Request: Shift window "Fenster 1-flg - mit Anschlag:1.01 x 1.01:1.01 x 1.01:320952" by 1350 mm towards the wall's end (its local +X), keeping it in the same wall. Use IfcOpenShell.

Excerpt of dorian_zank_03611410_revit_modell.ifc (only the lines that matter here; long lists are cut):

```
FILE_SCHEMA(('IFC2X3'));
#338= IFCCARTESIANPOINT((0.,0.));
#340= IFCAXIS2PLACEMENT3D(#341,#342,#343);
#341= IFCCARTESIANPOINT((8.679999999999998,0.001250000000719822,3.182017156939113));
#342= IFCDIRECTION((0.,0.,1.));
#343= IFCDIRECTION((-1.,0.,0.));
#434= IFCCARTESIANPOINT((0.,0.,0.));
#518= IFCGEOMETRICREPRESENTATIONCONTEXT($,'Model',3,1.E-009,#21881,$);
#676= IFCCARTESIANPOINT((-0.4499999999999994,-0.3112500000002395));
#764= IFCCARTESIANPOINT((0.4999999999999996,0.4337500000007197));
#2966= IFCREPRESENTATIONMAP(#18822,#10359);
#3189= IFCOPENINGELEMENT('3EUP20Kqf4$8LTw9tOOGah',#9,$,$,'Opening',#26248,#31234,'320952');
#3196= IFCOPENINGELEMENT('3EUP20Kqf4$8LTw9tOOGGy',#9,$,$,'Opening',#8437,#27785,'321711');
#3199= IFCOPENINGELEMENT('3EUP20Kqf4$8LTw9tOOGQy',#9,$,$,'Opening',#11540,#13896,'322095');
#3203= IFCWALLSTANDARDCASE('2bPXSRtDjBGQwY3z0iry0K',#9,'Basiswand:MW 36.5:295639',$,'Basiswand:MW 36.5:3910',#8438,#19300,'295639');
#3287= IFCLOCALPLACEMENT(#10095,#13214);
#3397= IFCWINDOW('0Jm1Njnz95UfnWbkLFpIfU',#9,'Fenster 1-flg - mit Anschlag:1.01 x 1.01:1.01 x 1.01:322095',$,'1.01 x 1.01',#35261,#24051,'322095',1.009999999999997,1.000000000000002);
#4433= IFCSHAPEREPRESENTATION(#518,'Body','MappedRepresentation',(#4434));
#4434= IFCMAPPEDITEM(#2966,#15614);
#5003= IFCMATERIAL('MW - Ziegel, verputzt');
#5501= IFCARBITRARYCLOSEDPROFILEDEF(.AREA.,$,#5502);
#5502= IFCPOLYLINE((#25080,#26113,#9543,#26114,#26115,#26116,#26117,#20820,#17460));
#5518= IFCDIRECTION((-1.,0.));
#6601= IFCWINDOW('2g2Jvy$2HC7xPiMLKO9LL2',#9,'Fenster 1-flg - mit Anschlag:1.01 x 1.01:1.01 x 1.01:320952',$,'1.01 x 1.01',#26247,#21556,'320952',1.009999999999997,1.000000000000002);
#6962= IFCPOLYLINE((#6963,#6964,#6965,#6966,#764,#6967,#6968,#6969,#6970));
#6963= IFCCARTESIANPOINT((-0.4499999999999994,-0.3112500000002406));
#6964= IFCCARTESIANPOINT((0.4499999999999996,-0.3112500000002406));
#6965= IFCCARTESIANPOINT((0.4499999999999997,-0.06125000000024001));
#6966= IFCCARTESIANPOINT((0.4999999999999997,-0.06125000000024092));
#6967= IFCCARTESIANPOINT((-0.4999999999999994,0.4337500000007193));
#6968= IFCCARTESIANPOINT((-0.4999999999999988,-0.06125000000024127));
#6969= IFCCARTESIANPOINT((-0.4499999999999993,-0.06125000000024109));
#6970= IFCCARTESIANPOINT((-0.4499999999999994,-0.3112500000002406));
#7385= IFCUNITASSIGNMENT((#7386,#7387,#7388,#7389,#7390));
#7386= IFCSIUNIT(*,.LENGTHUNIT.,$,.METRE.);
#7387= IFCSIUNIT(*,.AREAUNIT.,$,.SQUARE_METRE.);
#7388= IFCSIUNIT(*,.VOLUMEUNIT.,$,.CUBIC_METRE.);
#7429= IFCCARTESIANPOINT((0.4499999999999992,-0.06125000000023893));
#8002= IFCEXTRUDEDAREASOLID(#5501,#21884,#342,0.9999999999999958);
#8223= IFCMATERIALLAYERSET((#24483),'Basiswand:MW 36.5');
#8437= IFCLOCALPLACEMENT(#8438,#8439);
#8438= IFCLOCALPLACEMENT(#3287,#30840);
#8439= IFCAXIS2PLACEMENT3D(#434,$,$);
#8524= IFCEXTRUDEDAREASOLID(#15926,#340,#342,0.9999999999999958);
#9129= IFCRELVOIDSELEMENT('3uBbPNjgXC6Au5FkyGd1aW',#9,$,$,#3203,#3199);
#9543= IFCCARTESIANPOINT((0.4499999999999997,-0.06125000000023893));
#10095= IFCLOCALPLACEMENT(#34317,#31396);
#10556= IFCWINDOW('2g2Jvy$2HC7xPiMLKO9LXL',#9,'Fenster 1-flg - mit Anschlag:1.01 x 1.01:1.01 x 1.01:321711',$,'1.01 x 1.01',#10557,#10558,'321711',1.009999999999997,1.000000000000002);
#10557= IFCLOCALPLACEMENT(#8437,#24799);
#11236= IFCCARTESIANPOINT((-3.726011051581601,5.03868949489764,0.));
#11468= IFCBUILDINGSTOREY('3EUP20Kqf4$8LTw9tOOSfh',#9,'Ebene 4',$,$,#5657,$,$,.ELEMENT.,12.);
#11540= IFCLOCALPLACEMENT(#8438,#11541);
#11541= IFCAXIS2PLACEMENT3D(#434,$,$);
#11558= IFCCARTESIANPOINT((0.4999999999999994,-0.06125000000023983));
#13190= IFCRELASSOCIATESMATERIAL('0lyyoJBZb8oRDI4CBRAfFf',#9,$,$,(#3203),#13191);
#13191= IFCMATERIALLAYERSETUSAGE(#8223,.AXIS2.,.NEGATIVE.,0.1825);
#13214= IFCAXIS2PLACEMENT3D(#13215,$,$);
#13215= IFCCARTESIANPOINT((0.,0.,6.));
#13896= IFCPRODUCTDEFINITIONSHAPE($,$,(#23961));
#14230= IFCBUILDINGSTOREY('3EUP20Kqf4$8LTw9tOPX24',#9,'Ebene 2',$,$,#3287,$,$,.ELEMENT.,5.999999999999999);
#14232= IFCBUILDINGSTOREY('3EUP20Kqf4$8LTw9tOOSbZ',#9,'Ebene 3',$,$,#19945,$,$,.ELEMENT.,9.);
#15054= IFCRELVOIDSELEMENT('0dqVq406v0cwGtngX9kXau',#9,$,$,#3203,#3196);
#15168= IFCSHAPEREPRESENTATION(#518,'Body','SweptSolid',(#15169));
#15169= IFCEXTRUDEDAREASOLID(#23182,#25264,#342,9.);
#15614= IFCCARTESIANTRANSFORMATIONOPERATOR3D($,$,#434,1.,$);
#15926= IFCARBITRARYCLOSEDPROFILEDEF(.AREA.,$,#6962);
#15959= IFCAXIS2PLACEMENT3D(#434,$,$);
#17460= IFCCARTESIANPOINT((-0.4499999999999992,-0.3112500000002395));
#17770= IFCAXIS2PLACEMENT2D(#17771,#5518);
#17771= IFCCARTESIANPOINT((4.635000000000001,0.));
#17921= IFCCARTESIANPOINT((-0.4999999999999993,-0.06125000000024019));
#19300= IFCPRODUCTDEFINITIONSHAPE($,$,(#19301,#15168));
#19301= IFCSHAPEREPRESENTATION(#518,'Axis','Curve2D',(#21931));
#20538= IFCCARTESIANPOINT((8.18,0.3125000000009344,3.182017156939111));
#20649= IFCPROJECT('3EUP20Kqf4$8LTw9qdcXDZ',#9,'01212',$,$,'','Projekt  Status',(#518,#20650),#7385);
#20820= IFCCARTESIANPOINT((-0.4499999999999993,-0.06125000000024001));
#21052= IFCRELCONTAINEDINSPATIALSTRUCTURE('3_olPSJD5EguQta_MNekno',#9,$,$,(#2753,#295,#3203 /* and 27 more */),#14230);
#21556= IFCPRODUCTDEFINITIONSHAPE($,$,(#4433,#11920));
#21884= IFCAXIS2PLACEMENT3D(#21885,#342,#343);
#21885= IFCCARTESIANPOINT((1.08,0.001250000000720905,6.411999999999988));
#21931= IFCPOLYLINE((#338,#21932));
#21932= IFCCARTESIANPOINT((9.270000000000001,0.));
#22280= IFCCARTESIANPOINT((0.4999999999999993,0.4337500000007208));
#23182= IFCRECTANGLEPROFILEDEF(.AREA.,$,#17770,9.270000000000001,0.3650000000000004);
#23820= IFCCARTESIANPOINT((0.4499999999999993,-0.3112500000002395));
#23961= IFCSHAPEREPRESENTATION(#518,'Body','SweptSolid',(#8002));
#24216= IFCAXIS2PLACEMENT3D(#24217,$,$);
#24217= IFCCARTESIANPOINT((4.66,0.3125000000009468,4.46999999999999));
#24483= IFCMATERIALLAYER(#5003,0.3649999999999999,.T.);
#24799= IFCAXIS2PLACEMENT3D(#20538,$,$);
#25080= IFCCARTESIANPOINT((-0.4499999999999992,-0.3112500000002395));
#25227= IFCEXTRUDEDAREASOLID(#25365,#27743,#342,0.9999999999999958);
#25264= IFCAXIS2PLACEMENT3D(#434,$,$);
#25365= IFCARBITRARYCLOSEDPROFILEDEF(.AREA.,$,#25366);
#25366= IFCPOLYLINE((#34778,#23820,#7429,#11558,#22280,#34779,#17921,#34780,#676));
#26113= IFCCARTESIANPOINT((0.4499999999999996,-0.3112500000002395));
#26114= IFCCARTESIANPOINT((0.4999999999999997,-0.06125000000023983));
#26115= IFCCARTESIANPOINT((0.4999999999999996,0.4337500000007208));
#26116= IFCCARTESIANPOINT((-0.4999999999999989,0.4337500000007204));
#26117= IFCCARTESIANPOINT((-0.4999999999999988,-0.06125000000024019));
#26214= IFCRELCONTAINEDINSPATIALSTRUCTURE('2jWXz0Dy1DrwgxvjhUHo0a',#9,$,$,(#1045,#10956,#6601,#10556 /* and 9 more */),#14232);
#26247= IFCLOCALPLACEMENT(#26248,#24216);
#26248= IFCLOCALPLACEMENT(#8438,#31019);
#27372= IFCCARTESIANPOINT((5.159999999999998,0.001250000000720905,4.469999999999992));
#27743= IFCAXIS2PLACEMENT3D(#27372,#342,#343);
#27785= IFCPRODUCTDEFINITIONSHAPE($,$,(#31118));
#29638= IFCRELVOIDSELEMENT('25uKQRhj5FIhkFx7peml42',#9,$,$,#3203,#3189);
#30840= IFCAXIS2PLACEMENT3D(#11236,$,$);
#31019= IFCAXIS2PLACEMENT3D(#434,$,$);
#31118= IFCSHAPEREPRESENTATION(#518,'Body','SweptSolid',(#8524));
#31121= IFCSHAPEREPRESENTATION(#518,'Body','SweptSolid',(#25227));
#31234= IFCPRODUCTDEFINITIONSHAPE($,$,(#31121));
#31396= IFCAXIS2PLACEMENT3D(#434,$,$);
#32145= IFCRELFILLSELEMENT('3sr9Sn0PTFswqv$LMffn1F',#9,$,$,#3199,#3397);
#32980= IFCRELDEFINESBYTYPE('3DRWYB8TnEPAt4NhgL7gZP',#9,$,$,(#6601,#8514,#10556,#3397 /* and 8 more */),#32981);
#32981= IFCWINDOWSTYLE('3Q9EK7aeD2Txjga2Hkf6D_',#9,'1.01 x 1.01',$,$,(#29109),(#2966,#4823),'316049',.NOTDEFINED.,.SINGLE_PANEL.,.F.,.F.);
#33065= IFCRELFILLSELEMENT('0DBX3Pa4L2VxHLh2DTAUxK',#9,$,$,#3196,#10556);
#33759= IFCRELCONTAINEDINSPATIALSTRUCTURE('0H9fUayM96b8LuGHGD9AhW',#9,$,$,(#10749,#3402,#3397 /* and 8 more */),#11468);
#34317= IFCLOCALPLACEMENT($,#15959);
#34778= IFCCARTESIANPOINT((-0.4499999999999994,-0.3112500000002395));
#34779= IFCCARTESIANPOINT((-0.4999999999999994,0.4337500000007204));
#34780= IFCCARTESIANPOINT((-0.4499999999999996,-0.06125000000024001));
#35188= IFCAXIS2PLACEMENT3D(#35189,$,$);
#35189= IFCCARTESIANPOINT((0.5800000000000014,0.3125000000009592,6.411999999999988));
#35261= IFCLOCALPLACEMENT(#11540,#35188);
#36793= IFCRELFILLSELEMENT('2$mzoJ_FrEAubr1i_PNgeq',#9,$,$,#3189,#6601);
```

```python
import ifcopenshell
import ifcopenshell.api.geometry
import ifcopenshell.util.placement
import ifcopenshell.util.unit

model = ifcopenshell.open("dorian_zank_03611410_revit_modell.ifc")
unit_scale = ifcopenshell.util.unit.calculate_unit_scale(model)

window = model.by_guid("2g2Jvy$2HC7xPiMLKO9LL2")
opening = window.FillsVoids[0].RelatingOpeningElement
wall = opening.VoidsElements[0].RelatingBuildingElement

wall_matrix = ifcopenshell.util.placement.get_local_placement(wall.ObjectPlacement)
shift = wall_matrix[:3, 0] * 1.35 / unit_scale
before = ifcopenshell.util.placement.get_local_placement(window.ObjectPlacement)[:3, 3].copy()

# The window is placed relative to its opening, so it follows when the opening moves.
matrix = ifcopenshell.util.placement.get_local_placement(opening.ObjectPlacement)
matrix[:3, 3] += shift
ifcopenshell.api.geometry.edit_object_placement(
    model, product=opening, matrix=matrix, is_si=False, should_transform_children=True
)

after = ifcopenshell.util.placement.get_local_placement(window.ObjectPlacement)[:3, 3]
print("window moved by", (after - before).round(3) + 0.0)

model.write("dorian_zank_03611410_revit_modell-out.ifc")
```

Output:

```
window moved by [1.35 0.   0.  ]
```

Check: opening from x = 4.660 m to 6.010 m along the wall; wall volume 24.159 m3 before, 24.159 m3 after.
